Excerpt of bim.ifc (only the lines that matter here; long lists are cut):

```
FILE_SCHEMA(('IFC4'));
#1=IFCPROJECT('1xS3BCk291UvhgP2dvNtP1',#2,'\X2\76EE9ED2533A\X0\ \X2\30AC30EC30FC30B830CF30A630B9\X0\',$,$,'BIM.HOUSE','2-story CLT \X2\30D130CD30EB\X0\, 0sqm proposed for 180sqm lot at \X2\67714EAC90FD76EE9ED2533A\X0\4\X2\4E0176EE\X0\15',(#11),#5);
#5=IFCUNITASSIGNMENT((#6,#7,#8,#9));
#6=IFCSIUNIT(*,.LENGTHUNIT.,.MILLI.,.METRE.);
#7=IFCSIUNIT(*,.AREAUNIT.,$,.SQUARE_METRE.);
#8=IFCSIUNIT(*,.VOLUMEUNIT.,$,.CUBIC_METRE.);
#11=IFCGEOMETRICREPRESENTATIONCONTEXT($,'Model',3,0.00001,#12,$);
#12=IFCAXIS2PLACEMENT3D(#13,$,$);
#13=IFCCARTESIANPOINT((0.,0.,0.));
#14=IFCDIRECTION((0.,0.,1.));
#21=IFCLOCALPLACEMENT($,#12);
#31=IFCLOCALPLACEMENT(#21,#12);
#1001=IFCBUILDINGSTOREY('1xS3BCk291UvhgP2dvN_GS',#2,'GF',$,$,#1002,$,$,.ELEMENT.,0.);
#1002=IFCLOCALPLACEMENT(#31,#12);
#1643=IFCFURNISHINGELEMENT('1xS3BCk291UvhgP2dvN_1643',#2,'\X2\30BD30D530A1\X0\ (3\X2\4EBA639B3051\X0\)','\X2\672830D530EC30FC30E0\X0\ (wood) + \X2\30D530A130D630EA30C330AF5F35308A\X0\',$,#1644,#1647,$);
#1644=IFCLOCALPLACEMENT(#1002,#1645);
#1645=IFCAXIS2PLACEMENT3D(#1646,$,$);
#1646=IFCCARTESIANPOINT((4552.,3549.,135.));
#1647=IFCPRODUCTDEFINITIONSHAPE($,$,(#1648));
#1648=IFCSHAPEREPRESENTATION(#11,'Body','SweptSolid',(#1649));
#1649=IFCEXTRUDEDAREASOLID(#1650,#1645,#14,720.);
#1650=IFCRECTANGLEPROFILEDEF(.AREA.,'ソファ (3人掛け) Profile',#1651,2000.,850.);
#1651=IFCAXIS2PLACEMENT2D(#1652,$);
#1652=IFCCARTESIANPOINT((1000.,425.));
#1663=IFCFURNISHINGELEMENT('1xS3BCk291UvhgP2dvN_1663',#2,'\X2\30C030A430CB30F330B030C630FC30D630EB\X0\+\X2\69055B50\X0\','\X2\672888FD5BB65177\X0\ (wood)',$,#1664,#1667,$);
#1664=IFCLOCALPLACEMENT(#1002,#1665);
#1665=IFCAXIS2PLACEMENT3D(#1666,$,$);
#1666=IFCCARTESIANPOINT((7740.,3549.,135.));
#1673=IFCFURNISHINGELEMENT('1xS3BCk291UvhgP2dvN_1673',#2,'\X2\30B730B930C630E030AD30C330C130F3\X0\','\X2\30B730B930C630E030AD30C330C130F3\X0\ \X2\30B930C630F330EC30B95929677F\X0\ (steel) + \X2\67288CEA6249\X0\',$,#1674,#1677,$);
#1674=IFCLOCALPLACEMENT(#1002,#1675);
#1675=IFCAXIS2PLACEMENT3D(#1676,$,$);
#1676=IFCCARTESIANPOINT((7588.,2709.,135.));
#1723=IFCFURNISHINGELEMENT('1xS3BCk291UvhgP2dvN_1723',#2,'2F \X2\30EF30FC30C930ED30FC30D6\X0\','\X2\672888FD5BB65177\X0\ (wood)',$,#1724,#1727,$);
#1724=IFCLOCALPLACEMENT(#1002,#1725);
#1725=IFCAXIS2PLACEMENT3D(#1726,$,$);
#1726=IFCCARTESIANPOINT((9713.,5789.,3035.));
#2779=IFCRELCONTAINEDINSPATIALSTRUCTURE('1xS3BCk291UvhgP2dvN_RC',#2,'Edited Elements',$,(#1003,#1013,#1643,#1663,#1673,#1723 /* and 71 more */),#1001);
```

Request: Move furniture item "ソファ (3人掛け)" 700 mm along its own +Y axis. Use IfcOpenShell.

```python
import ifcopenshell
import ifcopenshell.api.geometry
import ifcopenshell.util.placement
import ifcopenshell.util.unit

model = ifcopenshell.open("bim.ifc")
unit_scale = ifcopenshell.util.unit.calculate_unit_scale(model)

item = model.by_guid("1xS3BCk291UvhgP2dvN_1643")
matrix = ifcopenshell.util.placement.get_local_placement(item.ObjectPlacement)
matrix[:3, 3] += matrix[:3, 1] * 0.7 / unit_scale
ifcopenshell.api.geometry.edit_object_placement(model, product=item, matrix=matrix, is_si=False)

print(ifcopenshell.util.placement.get_local_placement(item.ObjectPlacement).round(3) + 0.0)

model.write("bim-out.ifc")
```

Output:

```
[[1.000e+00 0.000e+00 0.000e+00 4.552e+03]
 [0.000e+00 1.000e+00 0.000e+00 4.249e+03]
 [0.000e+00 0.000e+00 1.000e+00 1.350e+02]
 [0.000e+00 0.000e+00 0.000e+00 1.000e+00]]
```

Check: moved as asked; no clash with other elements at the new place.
